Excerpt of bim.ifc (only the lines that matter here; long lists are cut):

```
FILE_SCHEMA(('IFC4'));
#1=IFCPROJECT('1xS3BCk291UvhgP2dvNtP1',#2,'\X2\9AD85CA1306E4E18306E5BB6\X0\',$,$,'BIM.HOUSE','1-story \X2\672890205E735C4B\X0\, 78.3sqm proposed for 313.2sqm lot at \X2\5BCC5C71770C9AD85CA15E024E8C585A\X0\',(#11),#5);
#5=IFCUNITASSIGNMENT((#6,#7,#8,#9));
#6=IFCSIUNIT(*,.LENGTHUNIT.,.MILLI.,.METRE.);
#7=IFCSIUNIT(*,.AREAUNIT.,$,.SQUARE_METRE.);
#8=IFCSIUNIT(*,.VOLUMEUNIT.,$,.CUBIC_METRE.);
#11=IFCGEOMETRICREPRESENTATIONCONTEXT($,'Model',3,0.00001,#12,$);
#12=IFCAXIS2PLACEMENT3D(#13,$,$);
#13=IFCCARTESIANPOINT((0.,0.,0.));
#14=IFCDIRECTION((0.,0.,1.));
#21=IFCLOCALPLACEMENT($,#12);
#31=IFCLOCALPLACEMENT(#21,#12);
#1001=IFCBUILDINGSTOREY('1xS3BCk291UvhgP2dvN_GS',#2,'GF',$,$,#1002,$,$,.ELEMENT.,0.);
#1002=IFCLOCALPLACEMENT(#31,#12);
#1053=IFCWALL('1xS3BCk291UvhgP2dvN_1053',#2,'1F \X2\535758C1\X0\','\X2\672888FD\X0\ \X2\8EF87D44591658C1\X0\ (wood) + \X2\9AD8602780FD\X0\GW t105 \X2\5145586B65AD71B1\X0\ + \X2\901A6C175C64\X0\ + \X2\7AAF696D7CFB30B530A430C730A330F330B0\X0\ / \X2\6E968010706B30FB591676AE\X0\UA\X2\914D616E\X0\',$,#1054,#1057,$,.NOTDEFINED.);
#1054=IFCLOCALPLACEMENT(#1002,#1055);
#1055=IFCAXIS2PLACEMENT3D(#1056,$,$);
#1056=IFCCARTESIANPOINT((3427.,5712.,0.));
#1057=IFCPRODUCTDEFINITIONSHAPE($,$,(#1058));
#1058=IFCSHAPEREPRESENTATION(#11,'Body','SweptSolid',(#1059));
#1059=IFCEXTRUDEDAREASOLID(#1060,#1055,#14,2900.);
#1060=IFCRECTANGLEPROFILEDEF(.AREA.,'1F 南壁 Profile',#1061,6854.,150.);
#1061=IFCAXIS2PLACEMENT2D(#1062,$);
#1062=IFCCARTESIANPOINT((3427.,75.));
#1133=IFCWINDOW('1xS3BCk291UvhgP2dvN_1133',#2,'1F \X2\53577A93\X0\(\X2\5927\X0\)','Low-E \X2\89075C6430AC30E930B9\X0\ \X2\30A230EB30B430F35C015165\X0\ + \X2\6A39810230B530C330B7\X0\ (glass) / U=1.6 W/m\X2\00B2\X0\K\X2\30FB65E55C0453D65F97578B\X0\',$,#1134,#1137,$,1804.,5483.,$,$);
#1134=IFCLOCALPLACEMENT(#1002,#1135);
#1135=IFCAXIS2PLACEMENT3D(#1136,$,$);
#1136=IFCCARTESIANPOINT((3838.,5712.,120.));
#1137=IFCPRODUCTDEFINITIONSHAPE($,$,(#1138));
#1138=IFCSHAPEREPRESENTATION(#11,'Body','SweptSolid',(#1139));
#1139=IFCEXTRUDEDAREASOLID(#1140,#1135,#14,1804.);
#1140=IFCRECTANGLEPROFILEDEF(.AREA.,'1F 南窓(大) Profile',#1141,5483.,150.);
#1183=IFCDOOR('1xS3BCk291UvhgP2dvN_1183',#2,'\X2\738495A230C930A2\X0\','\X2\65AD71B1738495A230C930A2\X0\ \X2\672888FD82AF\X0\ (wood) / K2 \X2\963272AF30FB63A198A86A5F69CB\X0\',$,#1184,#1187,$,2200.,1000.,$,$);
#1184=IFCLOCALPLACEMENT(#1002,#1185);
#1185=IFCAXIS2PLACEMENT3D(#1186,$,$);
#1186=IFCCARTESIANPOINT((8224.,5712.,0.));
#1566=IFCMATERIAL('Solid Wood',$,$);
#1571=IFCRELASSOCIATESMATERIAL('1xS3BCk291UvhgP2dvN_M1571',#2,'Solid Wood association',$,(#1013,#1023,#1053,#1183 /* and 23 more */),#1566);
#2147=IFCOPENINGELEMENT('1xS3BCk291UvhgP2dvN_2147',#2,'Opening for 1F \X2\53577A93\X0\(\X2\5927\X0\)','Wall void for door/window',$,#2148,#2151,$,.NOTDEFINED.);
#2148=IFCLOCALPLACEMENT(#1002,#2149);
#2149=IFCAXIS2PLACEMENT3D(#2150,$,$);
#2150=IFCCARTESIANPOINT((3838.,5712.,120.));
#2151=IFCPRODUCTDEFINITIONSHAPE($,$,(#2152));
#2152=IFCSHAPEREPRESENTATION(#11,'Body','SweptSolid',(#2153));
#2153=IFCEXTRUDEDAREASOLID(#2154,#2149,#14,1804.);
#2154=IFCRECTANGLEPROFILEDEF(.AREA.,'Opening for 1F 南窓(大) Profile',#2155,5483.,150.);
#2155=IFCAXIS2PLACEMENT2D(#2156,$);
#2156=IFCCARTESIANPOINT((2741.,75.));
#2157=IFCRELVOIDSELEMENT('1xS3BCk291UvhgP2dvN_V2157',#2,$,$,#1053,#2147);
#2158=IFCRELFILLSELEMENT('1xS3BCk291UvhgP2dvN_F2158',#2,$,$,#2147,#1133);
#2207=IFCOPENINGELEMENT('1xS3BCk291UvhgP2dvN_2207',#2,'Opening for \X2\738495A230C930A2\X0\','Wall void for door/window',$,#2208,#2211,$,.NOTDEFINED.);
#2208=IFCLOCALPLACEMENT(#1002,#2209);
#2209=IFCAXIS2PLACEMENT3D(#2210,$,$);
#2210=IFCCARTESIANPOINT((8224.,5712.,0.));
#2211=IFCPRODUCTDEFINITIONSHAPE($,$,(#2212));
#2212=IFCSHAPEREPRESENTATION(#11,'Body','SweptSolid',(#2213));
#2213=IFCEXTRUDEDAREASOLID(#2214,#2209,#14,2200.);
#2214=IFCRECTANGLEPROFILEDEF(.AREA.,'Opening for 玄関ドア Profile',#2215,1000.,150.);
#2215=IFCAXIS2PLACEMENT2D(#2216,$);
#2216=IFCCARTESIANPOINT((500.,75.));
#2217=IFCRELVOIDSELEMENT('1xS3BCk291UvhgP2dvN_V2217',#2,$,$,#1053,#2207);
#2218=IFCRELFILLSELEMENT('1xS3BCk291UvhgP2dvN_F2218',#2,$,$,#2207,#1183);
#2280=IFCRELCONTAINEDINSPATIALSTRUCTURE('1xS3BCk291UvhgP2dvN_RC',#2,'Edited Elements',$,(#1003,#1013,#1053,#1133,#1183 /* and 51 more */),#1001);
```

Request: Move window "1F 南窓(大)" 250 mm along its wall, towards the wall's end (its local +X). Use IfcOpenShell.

```python
import ifcopenshell
import ifcopenshell.api.geometry
import ifcopenshell.util.placement

model = ifcopenshell.open("bim.ifc")

window = model.by_guid("1xS3BCk291UvhgP2dvN_1133")
opening = window.FillsVoids[0].RelatingOpeningElement
wall = opening.VoidsElements[0].RelatingBuildingElement

wall_matrix = ifcopenshell.util.placement.get_local_placement(wall.ObjectPlacement)
shift = wall_matrix[:3, 0] * 250.0
before = ifcopenshell.util.placement.get_local_placement(window.ObjectPlacement)[:3, 3].copy()

# The window is not placed relative to its opening, so move both.
for product in (opening, window):
    matrix = ifcopenshell.util.placement.get_local_placement(product.ObjectPlacement)
    matrix[:3, 3] += shift
    ifcopenshell.api.geometry.edit_object_placement(model, product=product, matrix=matrix, is_si=False)

after = ifcopenshell.util.placement.get_local_placement(window.ObjectPlacement)[:3, 3]
print("window moved by", (after - before).round(3) + 0.0)

model.write("bim-out.ifc")
```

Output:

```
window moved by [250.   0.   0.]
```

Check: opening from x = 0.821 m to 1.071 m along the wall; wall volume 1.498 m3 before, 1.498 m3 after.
